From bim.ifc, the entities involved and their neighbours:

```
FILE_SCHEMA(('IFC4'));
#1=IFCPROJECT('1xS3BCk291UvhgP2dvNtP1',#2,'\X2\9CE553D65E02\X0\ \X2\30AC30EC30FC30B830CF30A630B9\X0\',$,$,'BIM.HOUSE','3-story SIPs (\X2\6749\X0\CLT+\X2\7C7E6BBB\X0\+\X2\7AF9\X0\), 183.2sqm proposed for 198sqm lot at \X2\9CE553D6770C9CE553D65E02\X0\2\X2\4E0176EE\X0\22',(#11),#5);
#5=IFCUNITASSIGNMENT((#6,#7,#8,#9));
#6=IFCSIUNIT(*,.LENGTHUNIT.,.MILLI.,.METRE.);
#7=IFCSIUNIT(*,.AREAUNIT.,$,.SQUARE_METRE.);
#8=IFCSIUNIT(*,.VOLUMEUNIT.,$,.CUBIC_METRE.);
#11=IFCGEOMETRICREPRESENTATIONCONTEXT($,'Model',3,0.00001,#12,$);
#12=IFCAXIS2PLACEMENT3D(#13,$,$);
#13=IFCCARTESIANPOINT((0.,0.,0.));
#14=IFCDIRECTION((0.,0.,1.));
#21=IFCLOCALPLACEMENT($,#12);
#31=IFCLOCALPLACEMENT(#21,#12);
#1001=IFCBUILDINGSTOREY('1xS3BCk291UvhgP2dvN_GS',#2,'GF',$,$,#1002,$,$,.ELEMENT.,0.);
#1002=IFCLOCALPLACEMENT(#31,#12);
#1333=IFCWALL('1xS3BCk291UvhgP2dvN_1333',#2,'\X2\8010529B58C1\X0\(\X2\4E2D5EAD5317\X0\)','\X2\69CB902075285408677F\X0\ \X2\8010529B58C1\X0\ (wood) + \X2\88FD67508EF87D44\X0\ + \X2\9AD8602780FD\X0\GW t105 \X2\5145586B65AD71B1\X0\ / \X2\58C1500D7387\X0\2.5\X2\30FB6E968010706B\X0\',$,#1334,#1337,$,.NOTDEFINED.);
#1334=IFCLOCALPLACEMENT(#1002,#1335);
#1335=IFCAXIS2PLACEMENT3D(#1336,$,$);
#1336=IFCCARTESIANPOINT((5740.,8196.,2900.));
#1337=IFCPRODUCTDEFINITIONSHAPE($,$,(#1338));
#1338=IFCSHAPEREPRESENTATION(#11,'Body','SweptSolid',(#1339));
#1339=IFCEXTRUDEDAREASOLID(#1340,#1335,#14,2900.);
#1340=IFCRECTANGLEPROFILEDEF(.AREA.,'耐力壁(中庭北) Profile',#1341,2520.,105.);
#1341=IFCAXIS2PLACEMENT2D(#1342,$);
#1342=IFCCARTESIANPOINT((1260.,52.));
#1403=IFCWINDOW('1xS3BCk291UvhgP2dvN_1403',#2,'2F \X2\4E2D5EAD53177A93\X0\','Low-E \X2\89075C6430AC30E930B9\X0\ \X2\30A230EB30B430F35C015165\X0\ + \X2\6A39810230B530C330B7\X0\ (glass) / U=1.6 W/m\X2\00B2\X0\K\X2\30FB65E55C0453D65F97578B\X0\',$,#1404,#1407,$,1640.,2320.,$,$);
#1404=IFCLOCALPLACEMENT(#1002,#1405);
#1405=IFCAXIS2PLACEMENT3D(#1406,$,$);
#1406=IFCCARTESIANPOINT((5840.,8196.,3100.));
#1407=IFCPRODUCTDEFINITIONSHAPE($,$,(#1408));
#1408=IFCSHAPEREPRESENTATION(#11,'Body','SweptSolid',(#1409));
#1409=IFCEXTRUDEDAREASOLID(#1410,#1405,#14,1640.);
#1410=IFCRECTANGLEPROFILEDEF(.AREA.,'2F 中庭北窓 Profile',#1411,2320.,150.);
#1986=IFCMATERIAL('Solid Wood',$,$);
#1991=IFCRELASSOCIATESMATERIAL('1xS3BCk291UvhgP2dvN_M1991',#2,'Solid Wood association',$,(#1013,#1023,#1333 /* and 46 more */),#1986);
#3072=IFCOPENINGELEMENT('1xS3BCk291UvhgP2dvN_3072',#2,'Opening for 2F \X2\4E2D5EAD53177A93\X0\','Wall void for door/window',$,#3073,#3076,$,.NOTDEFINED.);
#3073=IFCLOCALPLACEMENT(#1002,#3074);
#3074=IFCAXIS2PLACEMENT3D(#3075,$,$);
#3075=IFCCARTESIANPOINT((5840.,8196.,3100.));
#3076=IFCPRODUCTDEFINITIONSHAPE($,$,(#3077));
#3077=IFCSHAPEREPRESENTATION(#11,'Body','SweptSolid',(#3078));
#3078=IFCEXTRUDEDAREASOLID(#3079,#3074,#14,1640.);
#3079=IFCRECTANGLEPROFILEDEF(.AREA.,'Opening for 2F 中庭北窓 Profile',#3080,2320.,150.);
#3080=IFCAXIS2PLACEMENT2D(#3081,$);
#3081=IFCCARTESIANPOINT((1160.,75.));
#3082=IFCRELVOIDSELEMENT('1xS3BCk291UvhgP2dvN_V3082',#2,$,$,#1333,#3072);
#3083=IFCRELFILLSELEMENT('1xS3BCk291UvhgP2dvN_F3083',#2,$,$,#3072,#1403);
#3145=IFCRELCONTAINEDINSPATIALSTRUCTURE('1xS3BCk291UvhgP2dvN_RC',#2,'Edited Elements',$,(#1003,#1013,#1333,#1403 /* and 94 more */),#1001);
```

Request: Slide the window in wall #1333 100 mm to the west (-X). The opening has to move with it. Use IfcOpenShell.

```python
import ifcopenshell
import ifcopenshell.api.geometry
import ifcopenshell.util.placement
import ifcopenshell.util.unit

model = ifcopenshell.open("bim.ifc")
unit_scale = ifcopenshell.util.unit.calculate_unit_scale(model)

window = model.by_guid("1xS3BCk291UvhgP2dvN_1403")
opening = window.FillsVoids[0].RelatingOpeningElement
wall = opening.VoidsElements[0].RelatingBuildingElement

wall_matrix = ifcopenshell.util.placement.get_local_placement(wall.ObjectPlacement)
shift = wall_matrix[:3, 0] * -0.1 / unit_scale
before = ifcopenshell.util.placement.get_local_placement(window.ObjectPlacement)[:3, 3].copy()

# The window is not placed relative to its opening, so move both.
for product in (opening, window):
    matrix = ifcopenshell.util.placement.get_local_placement(product.ObjectPlacement)
    matrix[:3, 3] += shift
    ifcopenshell.api.geometry.edit_object_placement(model, product=product, matrix=matrix, is_si=False)

after = ifcopenshell.util.placement.get_local_placement(window.ObjectPlacement)[:3, 3]
print("window moved by", (after - before).round(3) + 0.0)

model.write("bim_updated.ifc")
```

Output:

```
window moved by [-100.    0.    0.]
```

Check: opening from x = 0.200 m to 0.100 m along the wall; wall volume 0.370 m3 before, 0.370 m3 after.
